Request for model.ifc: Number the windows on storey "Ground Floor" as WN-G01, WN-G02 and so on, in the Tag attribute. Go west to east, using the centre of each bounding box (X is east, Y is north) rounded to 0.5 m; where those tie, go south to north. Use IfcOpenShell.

First a look at what the model holds.

```python
import ifcopenshell
import ifcopenshell.util.element
import ifcopenshell.util.placement

model = ifcopenshell.open("model.ifc")
print(model.schema)
storey = next(s for s in model.by_type("IfcBuildingStorey") if s.Name == "Ground Floor")
windows = [e for e in ifcopenshell.util.element.get_decomposition(storey) if e.is_a("IfcWindow")]
for e in sorted(windows, key=lambda e: e.id()):
    origin = ifcopenshell.util.placement.get_local_placement(e.ObjectPlacement)[:3, 3]
    print(e.id(), e.Tag, e.Name, origin.round(2) + 0.0, sep=" | ")
```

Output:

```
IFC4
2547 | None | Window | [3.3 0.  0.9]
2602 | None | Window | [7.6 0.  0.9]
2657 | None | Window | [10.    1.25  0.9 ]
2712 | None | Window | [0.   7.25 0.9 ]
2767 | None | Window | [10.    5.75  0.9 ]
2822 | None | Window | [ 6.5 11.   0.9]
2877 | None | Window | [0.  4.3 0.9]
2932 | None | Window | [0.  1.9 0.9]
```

```python
import ifcopenshell
import ifcopenshell.geom
import ifcopenshell.util.element
import ifcopenshell.util.shape

model = ifcopenshell.open("model.ifc")
settings = ifcopenshell.geom.settings()
settings.set("use-world-coords", True)


def centre(element):
    shape = ifcopenshell.geom.create_shape(settings, element)
    return ifcopenshell.util.shape.get_bbox_centroid(shape.geometry)


storey = next(s for s in model.by_type("IfcBuildingStorey") if s.Name == "Ground Floor")
windows = [e for e in ifcopenshell.util.element.get_decomposition(storey) if e.is_a("IfcWindow")]

# Insertion points can sit at a corner or the storey origin, so sort by the geometry (in metres).
centres = {e: centre(e) for e in windows}
windows.sort(key=lambda e: (round(centres[e][0] / 0.5), centres[e][1]))

for i, e in enumerate(windows, start=1):
    number = f"WN-G{i:02d}"
    e.Tag = number
    print(e.id(), number)

model.write("model_v2.ifc")
```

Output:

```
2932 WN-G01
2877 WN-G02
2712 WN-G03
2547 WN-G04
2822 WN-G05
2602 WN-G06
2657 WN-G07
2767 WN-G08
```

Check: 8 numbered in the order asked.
